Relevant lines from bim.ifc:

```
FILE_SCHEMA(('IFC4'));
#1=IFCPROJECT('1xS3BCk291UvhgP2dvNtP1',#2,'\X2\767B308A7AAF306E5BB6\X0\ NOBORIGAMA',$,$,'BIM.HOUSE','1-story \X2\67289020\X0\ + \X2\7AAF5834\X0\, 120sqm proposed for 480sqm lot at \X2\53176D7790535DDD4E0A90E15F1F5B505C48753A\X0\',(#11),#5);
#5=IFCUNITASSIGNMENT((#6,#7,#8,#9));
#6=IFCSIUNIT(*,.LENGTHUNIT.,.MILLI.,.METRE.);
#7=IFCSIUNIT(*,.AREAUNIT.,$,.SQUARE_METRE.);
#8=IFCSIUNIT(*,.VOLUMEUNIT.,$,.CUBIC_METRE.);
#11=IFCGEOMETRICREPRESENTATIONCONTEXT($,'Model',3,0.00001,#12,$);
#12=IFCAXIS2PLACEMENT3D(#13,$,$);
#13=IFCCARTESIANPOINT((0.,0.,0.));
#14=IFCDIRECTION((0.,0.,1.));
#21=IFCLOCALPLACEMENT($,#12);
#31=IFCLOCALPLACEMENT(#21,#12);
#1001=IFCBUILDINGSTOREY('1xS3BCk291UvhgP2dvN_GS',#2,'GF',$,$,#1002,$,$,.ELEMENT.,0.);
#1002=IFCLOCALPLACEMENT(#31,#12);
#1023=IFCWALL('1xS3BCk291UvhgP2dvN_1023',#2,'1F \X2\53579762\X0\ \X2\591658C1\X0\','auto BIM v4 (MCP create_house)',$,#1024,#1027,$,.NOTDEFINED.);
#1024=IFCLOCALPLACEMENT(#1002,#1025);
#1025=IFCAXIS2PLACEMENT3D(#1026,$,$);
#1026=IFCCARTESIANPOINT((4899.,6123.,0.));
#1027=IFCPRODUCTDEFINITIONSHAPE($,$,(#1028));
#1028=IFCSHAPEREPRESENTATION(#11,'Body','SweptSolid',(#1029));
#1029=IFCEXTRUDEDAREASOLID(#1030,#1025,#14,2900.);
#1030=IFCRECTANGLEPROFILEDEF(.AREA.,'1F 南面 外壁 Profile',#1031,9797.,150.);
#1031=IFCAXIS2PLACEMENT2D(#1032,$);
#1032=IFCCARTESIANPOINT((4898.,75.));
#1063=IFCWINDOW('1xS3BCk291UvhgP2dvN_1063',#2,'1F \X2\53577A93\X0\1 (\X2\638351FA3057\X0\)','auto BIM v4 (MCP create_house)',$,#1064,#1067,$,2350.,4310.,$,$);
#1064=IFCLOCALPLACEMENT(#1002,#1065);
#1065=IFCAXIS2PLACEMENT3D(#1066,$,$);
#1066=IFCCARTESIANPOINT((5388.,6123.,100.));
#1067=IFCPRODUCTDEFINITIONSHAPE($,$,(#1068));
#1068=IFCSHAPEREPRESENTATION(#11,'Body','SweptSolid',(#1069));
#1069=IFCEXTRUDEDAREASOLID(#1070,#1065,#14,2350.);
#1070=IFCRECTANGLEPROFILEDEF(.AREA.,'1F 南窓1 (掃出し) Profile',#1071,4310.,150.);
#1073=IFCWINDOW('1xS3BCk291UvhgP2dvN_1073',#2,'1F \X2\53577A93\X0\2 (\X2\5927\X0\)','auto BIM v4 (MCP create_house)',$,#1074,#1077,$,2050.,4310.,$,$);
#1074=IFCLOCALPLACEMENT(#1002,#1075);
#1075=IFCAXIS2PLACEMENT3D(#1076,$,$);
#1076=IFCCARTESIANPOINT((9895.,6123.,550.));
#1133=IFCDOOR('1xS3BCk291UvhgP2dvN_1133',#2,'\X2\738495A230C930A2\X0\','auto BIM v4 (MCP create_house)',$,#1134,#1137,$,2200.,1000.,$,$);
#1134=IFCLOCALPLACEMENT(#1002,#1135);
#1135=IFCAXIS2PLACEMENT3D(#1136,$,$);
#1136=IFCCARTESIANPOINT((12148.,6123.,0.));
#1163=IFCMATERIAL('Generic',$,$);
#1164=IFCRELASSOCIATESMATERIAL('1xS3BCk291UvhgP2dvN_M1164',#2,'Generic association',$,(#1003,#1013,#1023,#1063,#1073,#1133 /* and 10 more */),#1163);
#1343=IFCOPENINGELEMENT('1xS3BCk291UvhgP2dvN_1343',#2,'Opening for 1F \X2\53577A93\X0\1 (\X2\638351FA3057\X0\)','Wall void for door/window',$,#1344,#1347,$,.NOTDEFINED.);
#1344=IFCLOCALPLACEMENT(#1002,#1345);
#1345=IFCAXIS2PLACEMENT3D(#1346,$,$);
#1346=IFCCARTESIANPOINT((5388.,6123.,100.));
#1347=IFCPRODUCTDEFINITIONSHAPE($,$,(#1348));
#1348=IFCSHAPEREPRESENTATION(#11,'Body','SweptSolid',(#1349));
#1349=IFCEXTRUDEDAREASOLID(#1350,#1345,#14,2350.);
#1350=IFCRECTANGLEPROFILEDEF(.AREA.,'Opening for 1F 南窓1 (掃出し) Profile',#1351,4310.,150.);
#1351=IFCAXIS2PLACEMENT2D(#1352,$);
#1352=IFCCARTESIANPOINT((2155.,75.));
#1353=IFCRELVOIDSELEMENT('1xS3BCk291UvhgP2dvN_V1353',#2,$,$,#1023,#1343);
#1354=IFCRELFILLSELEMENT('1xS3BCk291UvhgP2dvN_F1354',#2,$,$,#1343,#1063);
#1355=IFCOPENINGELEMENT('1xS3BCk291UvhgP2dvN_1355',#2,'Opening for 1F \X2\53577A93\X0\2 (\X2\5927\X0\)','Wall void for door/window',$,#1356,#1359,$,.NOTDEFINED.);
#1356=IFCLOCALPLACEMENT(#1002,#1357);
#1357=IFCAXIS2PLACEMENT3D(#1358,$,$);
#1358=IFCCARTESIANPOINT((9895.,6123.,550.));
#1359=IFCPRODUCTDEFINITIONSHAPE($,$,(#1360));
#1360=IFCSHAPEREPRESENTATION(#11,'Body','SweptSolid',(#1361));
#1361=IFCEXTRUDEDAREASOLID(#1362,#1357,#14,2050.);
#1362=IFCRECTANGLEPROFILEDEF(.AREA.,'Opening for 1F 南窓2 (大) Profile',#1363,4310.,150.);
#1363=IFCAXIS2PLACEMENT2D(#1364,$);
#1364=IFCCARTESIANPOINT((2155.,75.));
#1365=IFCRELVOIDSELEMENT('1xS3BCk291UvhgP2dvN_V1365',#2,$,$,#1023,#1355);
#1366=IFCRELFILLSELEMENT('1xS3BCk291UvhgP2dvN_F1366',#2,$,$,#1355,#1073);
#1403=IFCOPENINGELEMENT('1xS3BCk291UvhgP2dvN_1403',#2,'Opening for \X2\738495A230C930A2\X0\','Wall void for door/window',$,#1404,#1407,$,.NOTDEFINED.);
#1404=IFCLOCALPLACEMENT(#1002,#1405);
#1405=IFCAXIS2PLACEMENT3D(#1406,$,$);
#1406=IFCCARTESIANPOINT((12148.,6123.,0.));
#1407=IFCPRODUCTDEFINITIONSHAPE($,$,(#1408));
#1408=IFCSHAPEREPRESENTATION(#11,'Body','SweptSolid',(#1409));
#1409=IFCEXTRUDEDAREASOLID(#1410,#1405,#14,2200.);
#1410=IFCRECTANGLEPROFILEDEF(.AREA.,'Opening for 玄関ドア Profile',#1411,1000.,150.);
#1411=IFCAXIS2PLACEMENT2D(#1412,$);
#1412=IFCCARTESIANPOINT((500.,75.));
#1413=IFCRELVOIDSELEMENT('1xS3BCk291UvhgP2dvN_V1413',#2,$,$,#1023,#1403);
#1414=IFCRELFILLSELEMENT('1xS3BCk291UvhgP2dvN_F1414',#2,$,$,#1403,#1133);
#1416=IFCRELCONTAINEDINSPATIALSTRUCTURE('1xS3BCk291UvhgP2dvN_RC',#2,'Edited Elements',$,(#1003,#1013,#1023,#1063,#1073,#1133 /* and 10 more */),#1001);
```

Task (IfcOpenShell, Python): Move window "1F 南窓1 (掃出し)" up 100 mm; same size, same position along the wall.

```python
import numpy as np
import ifcopenshell
import ifcopenshell.api.geometry
import ifcopenshell.util.placement
import ifcopenshell.util.unit

model = ifcopenshell.open("bim.ifc")
unit_scale = ifcopenshell.util.unit.calculate_unit_scale(model)

window = model.by_guid("1xS3BCk291UvhgP2dvN_1063")
opening = window.FillsVoids[0].RelatingOpeningElement
dz = 100.0

shift = np.array([0.0, 0.0, dz])
# The window is not placed relative to its opening, so move both.
for product in (opening, window):
    matrix = ifcopenshell.util.placement.get_local_placement(product.ObjectPlacement)
    matrix[:3, 3] += shift
    ifcopenshell.api.geometry.edit_object_placement(model, product=product, matrix=matrix, is_si=False)

print(f"moved by {dz * unit_scale:+.3f} m")

model.write("bim-out.ifc")
```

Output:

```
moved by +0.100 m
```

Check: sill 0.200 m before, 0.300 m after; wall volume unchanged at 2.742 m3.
